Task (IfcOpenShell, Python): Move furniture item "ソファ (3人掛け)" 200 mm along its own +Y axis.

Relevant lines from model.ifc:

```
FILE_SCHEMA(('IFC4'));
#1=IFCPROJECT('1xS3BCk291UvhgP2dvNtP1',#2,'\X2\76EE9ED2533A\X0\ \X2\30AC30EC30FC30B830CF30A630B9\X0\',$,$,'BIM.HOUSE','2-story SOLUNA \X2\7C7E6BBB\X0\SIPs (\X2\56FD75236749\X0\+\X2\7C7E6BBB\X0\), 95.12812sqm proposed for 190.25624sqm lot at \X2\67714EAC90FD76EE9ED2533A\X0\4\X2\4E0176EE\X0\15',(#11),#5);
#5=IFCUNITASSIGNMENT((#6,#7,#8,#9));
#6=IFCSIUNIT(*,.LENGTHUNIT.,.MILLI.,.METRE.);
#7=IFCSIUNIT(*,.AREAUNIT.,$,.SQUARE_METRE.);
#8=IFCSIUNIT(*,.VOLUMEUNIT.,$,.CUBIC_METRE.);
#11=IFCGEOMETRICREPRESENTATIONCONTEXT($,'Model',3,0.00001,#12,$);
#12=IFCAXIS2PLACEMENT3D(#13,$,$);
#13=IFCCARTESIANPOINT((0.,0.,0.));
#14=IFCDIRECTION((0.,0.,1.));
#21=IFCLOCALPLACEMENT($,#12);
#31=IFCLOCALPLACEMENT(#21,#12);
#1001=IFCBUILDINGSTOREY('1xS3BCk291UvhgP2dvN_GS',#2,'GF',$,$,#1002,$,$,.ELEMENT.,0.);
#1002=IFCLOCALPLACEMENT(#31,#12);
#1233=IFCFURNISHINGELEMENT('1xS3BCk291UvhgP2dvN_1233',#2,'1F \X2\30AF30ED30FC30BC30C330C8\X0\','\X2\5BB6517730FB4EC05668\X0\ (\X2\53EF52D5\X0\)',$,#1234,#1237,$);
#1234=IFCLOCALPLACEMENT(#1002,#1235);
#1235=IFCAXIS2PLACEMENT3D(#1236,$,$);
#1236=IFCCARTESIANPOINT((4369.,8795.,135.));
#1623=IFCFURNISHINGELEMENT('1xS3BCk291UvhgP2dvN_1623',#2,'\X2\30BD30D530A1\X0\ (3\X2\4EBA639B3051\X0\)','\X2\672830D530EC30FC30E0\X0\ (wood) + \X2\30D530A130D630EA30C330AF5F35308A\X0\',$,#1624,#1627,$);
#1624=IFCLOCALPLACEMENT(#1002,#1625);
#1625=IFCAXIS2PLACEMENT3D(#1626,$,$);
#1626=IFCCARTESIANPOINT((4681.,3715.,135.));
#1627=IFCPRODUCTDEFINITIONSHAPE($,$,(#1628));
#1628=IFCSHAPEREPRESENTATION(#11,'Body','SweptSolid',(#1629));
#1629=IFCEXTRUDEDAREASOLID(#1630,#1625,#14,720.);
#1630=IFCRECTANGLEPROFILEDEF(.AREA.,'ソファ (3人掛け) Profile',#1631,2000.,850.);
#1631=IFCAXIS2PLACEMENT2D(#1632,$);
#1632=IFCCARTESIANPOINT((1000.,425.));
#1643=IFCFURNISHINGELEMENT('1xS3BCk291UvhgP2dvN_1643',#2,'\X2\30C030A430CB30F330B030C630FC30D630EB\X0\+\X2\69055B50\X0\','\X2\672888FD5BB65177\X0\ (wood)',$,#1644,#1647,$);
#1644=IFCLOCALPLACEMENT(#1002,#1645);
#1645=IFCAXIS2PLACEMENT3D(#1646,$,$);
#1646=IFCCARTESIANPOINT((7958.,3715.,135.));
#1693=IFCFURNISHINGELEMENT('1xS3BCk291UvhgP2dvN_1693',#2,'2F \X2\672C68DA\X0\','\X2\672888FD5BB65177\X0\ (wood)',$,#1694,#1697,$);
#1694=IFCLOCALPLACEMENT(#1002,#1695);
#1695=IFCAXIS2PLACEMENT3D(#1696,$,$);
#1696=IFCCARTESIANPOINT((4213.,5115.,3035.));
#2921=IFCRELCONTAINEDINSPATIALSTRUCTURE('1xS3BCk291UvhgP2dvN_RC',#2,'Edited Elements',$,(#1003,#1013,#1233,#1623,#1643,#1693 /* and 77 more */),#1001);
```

```python
import ifcopenshell
import ifcopenshell.api.geometry
import ifcopenshell.util.placement
import ifcopenshell.util.unit

model = ifcopenshell.open("model.ifc")
unit_scale = ifcopenshell.util.unit.calculate_unit_scale(model)

item = model.by_guid("1xS3BCk291UvhgP2dvN_1623")
matrix = ifcopenshell.util.placement.get_local_placement(item.ObjectPlacement)
matrix[:3, 3] += matrix[:3, 1] * 0.2 / unit_scale
ifcopenshell.api.geometry.edit_object_placement(model, product=item, matrix=matrix, is_si=False)

print(ifcopenshell.util.placement.get_local_placement(item.ObjectPlacement).round(3) + 0.0)

model.write("model_edited.ifc")
```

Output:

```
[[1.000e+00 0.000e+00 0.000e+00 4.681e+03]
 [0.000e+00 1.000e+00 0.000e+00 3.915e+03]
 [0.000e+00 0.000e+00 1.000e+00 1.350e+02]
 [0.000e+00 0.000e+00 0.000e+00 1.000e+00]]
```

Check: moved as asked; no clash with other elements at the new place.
